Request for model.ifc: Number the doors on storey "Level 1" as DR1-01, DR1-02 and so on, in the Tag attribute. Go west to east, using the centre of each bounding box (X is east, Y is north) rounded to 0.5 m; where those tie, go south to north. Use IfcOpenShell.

First a look at what the model holds.

```python
import ifcopenshell
import ifcopenshell.util.element
import ifcopenshell.util.placement

model = ifcopenshell.open("model.ifc")
print(model.schema)
storey = next(s for s in model.by_type("IfcBuildingStorey") if s.Name == "Level 1")
doors = [e for e in ifcopenshell.util.element.get_decomposition(storey) if e.is_a("IfcDoor")]
for e in sorted(doors, key=lambda e: e.id()):
    origin = ifcopenshell.util.placement.get_local_placement(e.ObjectPlacement)[:3, 3]
    print(e.id(), e.Tag, e.Name, origin.round(2) + 0.0, sep=" | ")
```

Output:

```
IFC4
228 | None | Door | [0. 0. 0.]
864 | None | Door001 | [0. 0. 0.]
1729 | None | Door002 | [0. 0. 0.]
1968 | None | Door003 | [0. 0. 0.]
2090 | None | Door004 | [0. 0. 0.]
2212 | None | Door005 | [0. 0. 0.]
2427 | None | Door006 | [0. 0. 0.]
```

```python
import ifcopenshell
import ifcopenshell.geom
import ifcopenshell.util.element
import ifcopenshell.util.shape

model = ifcopenshell.open("model.ifc")
settings = ifcopenshell.geom.settings()
settings.set("use-world-coords", True)


def centre(element):
    shape = ifcopenshell.geom.create_shape(settings, element)
    return ifcopenshell.util.shape.get_bbox_centroid(shape.geometry)


storey = next(s for s in model.by_type("IfcBuildingStorey") if s.Name == "Level 1")
doors = [e for e in ifcopenshell.util.element.get_decomposition(storey) if e.is_a("IfcDoor")]

# Insertion points can sit at a corner or the storey origin, so sort by the geometry (in metres).
centres = {e: centre(e) for e in doors}
doors.sort(key=lambda e: (round(centres[e][0] / 0.5), centres[e][1]))

for i, e in enumerate(doors, start=1):
    number = f"DR1-{i:02d}"
    e.Tag = number
    print(e.id(), number)

model.write("model_v2.ifc")
```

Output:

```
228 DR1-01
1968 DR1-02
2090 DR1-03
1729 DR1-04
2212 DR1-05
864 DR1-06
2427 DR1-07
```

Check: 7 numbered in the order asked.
